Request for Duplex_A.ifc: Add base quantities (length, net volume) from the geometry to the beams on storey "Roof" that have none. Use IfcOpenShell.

First a look at what the model holds.

```python
import ifcopenshell
import ifcopenshell.util.element
import ifcopenshell.util.unit

model = ifcopenshell.open("Duplex_A.ifc")
print(model.schema)
for unit_type in ("LENGTHUNIT", "AREAUNIT", "VOLUMEUNIT"):
    print(unit_type, ifcopenshell.util.unit.calculate_unit_scale(model, unit_type))
storey = next(s for s in model.by_type("IfcBuildingStorey") if s.Name == "Roof")
beams = [e for e in ifcopenshell.util.element.get_decomposition(storey) if e.is_a("IfcBeam")]
for e in sorted(beams, key=lambda e: e.id()):
    print(e.id(), e.is_a(), e.Name, list(ifcopenshell.util.element.get_psets(e, qtos_only=True)), sep=" | ")
```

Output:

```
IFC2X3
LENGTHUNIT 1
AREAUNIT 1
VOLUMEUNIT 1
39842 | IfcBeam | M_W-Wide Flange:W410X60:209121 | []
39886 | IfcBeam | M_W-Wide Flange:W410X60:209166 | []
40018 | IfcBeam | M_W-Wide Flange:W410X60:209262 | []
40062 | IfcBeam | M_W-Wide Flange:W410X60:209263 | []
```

```python
import ifcopenshell
import ifcopenshell.api.pset
import ifcopenshell.geom
import ifcopenshell.util.element
import ifcopenshell.util.shape
import ifcopenshell.util.unit

model = ifcopenshell.open("Duplex_A.ifc")
unit_scale = ifcopenshell.util.unit.calculate_unit_scale(model)
volume_scale = ifcopenshell.util.unit.calculate_unit_scale(model, "VOLUMEUNIT")
settings = ifcopenshell.geom.settings()

storey = next(s for s in model.by_type("IfcBuildingStorey") if s.Name == "Roof")
beams = [e for e in ifcopenshell.util.element.get_decomposition(storey) if e.is_a("IfcBeam")]

for e in sorted(beams, key=lambda e: e.id()):
    if ifcopenshell.util.element.get_psets(e, qtos_only=True, should_inherit=False):
        continue
    # Geometry comes back in metres, in the element's own axes.
    shape = ifcopenshell.geom.create_shape(settings, e)
    values = {
        "Length": ifcopenshell.util.shape.get_max_xyz(shape.geometry) / unit_scale,
        "NetVolume": ifcopenshell.util.shape.get_volume(shape.geometry) / volume_scale,
    }
    qto = ifcopenshell.api.pset.add_qto(model, product=e, name="BaseQuantities")
    ifcopenshell.api.pset.edit_qto(model, qto=qto, properties=values)
    print(e.id(), {k: round(v, 3) for k, v in values.items()})

model.write("Duplex_A_v2.ifc")
```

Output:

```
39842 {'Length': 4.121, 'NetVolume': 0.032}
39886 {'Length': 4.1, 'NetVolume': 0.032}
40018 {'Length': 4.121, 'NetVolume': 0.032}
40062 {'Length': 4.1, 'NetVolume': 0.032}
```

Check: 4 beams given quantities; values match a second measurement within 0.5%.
